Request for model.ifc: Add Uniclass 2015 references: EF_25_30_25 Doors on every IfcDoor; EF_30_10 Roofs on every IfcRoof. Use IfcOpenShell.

First a look at what the model holds.

```python
import ifcopenshell

model = ifcopenshell.open("model.ifc")
print(model.schema)
print("classifications:", [c.Name for c in model.by_type("IfcClassification")])
for ifc_class in ("IfcDoor", "IfcRoof", "IfcStair", "IfcWall", "IfcWindow"):
    print(ifc_class, len(model.by_type(ifc_class)))
```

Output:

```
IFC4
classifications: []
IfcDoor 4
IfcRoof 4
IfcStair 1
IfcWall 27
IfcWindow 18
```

```python
import ifcopenshell
import ifcopenshell.api.classification

model = ifcopenshell.open("model.ifc")

system = ifcopenshell.api.classification.add_classification(model, classification="Uniclass 2015")

codes = {
    "IfcDoor": ("EF_25_30_25", "Doors"),
    "IfcRoof": ("EF_30_10", "Roofs"),
}
for ifc_class, (code, name) in codes.items():
    products = model.by_type(ifc_class)
    ifcopenshell.api.classification.add_reference(
        model, products=products, classification=system, identification=code, name=name
    )
    print(code, len(products))

model.write("model-out.ifc")
```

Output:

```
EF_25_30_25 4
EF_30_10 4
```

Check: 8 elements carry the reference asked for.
